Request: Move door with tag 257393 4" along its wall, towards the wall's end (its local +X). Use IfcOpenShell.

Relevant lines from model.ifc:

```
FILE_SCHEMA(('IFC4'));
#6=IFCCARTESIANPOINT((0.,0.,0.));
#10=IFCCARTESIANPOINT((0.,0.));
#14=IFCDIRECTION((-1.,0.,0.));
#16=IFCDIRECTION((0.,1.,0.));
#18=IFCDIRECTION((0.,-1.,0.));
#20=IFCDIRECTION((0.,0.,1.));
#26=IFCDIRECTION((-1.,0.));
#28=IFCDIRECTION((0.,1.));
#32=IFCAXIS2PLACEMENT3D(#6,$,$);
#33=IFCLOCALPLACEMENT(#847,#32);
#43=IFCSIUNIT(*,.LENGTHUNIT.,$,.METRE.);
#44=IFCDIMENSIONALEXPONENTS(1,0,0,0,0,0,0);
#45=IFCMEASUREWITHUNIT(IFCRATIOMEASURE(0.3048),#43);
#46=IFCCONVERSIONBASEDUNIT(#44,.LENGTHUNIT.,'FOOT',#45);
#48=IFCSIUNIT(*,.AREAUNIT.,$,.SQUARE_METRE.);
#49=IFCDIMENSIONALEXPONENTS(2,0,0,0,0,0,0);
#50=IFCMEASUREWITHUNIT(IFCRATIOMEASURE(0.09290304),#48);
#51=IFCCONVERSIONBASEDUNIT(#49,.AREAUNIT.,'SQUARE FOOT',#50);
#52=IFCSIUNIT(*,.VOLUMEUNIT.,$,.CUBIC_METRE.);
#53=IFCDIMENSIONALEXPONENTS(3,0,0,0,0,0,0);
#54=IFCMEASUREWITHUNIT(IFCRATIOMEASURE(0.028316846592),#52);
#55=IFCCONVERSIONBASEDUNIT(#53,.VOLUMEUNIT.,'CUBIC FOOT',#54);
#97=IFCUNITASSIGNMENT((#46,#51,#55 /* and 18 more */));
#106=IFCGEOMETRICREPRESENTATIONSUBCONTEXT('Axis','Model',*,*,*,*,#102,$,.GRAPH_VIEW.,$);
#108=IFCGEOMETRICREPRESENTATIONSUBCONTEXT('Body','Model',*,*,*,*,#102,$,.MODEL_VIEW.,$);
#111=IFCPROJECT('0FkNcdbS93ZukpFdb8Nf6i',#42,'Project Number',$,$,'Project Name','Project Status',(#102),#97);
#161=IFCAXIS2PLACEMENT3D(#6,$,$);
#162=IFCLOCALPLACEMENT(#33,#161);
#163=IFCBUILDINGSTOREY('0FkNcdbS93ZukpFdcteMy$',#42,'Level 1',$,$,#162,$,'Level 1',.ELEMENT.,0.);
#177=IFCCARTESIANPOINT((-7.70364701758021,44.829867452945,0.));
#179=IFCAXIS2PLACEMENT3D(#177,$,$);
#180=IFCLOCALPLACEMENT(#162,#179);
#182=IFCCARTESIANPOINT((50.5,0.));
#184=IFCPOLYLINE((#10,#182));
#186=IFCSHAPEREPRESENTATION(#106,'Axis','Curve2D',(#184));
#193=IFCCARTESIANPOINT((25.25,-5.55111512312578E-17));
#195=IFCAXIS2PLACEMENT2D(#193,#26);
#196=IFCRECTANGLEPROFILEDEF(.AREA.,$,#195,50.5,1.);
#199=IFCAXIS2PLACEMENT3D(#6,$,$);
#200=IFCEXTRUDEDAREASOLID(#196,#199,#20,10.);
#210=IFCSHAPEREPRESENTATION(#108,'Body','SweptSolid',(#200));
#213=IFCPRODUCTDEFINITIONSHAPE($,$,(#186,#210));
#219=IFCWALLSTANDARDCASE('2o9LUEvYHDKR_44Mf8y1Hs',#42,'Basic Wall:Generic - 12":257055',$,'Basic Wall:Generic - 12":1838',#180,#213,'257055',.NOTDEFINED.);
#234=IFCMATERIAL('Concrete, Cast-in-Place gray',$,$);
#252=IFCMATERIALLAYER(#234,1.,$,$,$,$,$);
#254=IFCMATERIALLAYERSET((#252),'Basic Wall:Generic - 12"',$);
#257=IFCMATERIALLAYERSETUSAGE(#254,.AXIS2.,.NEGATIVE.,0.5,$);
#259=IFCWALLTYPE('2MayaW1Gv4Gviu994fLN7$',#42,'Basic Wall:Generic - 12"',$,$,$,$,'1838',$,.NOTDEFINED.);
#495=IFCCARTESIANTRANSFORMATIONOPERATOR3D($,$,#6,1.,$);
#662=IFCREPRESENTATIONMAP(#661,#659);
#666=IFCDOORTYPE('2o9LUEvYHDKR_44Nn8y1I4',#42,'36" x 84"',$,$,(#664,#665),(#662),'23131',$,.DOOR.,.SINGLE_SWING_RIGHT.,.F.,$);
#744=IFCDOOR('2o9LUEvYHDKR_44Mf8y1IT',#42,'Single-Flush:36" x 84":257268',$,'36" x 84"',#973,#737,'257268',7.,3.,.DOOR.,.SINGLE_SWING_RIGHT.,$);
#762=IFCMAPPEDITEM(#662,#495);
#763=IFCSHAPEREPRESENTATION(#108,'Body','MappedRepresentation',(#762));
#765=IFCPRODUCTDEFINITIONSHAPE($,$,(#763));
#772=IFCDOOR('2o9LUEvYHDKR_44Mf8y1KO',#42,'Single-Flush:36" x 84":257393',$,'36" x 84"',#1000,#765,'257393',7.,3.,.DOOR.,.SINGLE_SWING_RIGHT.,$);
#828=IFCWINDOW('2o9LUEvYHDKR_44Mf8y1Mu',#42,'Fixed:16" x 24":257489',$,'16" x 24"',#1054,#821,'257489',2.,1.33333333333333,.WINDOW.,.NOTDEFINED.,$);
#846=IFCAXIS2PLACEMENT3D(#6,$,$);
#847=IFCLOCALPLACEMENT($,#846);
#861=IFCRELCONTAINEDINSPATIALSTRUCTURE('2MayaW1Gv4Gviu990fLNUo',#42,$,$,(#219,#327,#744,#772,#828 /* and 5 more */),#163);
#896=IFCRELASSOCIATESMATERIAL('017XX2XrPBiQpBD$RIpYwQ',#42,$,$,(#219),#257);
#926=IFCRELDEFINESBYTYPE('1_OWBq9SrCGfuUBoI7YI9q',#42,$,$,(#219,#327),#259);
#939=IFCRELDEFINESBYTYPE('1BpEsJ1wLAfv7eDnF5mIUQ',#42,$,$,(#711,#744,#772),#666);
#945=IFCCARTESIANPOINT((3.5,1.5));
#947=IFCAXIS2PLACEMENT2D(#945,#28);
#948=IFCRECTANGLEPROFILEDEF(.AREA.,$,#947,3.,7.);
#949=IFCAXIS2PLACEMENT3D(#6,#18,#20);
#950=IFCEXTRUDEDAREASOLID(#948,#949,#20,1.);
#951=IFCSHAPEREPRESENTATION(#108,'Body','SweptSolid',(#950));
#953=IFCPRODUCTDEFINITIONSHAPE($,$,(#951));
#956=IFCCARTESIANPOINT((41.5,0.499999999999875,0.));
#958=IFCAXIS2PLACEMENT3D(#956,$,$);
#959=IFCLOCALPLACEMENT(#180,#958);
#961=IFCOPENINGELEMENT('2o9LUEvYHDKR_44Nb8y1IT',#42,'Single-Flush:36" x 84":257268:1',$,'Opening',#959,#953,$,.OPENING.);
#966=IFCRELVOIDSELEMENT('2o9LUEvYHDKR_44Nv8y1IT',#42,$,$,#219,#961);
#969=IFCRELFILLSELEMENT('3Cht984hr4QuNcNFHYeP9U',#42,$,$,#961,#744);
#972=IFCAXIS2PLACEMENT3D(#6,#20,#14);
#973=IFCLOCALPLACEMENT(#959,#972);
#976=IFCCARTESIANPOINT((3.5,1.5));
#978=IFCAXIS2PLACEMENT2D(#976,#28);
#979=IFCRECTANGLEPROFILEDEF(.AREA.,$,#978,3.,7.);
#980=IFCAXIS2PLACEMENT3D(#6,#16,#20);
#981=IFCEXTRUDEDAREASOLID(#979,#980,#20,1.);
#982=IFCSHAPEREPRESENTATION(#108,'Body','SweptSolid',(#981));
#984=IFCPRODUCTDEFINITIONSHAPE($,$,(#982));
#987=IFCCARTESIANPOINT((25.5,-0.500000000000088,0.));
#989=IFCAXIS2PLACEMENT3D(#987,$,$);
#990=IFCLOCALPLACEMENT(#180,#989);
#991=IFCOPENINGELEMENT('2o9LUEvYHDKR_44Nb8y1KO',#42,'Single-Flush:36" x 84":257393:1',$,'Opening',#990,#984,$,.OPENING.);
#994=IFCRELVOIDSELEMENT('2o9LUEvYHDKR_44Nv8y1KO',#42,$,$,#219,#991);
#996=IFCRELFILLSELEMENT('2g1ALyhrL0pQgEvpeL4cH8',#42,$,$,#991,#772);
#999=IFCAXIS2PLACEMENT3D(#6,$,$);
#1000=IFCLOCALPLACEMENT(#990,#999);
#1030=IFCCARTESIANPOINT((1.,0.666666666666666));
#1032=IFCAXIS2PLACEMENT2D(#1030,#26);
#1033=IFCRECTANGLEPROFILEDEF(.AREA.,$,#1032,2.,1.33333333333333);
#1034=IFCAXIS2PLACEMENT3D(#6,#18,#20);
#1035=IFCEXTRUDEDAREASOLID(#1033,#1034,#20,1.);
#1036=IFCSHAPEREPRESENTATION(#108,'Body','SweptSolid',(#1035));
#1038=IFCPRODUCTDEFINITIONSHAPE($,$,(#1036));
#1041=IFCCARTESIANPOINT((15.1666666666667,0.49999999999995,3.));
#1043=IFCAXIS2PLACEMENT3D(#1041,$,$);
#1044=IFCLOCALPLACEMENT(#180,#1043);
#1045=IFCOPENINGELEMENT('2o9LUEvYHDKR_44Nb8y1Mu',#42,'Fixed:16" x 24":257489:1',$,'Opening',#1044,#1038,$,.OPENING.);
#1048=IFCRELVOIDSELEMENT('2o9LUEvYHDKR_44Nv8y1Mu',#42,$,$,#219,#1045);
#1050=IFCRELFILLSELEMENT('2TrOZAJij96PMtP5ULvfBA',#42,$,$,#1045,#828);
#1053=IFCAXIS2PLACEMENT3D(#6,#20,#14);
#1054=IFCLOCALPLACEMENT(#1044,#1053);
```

```python
import ifcopenshell
import ifcopenshell.api.geometry
import ifcopenshell.util.placement
import ifcopenshell.util.unit

model = ifcopenshell.open("model.ifc")
unit_scale = ifcopenshell.util.unit.calculate_unit_scale(model)

door = model.by_id(772)
opening = door.FillsVoids[0].RelatingOpeningElement
wall = opening.VoidsElements[0].RelatingBuildingElement

wall_matrix = ifcopenshell.util.placement.get_local_placement(wall.ObjectPlacement)
shift = wall_matrix[:3, 0] * 4 * 0.0254 / unit_scale
before = ifcopenshell.util.placement.get_local_placement(door.ObjectPlacement)[:3, 3].copy()

# The door is placed relative to its opening, so it follows when the opening moves.
matrix = ifcopenshell.util.placement.get_local_placement(opening.ObjectPlacement)
matrix[:3, 3] += shift
ifcopenshell.api.geometry.edit_object_placement(
    model, product=opening, matrix=matrix, is_si=False, should_transform_children=True
)

after = ifcopenshell.util.placement.get_local_placement(door.ObjectPlacement)[:3, 3]
print("door moved by", (after - before).round(3) + 0.0)

model.write("model-out.ifc")
```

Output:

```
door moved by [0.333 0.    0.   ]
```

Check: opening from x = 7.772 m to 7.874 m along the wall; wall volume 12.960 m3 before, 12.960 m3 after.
